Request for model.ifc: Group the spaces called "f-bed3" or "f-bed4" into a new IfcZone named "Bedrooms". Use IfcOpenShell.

First a look at what the model holds.

```python
import ifcopenshell

model = ifcopenshell.open("model.ifc")
print(model.schema)
seen = {}
for space in model.by_type("IfcSpace"):
    seen[space.LongName] = seen.get(space.LongName, 0) + 1
for name, count in sorted(seen.items(), key=str):
    print(count, "x", name)
print("zones:", [z.Name for z in model.by_type("IfcZone")][:20])
```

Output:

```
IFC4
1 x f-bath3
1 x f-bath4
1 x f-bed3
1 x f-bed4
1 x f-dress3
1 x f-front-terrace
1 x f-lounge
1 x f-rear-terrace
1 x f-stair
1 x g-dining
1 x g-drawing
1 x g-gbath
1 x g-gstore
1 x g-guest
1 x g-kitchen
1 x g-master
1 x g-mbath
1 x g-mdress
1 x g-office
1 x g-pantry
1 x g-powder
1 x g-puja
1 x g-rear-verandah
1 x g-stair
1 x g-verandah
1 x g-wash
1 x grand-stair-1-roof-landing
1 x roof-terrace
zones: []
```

```python
import ifcopenshell
import ifcopenshell.api.group
import ifcopenshell.api.root

model = ifcopenshell.open("model.ifc")

names = {"f-bed3", "f-bed4"}
spaces = [s for s in model.by_type("IfcSpace") if s.LongName in names]

zone = ifcopenshell.api.root.create_entity(model, ifc_class="IfcZone", name="Bedrooms")
ifcopenshell.api.group.assign_group(model, products=spaces, group=zone)
print(len(spaces), "spaces in", zone.Name)

model.write("model_edited.ifc")
```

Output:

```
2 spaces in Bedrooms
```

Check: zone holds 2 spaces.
